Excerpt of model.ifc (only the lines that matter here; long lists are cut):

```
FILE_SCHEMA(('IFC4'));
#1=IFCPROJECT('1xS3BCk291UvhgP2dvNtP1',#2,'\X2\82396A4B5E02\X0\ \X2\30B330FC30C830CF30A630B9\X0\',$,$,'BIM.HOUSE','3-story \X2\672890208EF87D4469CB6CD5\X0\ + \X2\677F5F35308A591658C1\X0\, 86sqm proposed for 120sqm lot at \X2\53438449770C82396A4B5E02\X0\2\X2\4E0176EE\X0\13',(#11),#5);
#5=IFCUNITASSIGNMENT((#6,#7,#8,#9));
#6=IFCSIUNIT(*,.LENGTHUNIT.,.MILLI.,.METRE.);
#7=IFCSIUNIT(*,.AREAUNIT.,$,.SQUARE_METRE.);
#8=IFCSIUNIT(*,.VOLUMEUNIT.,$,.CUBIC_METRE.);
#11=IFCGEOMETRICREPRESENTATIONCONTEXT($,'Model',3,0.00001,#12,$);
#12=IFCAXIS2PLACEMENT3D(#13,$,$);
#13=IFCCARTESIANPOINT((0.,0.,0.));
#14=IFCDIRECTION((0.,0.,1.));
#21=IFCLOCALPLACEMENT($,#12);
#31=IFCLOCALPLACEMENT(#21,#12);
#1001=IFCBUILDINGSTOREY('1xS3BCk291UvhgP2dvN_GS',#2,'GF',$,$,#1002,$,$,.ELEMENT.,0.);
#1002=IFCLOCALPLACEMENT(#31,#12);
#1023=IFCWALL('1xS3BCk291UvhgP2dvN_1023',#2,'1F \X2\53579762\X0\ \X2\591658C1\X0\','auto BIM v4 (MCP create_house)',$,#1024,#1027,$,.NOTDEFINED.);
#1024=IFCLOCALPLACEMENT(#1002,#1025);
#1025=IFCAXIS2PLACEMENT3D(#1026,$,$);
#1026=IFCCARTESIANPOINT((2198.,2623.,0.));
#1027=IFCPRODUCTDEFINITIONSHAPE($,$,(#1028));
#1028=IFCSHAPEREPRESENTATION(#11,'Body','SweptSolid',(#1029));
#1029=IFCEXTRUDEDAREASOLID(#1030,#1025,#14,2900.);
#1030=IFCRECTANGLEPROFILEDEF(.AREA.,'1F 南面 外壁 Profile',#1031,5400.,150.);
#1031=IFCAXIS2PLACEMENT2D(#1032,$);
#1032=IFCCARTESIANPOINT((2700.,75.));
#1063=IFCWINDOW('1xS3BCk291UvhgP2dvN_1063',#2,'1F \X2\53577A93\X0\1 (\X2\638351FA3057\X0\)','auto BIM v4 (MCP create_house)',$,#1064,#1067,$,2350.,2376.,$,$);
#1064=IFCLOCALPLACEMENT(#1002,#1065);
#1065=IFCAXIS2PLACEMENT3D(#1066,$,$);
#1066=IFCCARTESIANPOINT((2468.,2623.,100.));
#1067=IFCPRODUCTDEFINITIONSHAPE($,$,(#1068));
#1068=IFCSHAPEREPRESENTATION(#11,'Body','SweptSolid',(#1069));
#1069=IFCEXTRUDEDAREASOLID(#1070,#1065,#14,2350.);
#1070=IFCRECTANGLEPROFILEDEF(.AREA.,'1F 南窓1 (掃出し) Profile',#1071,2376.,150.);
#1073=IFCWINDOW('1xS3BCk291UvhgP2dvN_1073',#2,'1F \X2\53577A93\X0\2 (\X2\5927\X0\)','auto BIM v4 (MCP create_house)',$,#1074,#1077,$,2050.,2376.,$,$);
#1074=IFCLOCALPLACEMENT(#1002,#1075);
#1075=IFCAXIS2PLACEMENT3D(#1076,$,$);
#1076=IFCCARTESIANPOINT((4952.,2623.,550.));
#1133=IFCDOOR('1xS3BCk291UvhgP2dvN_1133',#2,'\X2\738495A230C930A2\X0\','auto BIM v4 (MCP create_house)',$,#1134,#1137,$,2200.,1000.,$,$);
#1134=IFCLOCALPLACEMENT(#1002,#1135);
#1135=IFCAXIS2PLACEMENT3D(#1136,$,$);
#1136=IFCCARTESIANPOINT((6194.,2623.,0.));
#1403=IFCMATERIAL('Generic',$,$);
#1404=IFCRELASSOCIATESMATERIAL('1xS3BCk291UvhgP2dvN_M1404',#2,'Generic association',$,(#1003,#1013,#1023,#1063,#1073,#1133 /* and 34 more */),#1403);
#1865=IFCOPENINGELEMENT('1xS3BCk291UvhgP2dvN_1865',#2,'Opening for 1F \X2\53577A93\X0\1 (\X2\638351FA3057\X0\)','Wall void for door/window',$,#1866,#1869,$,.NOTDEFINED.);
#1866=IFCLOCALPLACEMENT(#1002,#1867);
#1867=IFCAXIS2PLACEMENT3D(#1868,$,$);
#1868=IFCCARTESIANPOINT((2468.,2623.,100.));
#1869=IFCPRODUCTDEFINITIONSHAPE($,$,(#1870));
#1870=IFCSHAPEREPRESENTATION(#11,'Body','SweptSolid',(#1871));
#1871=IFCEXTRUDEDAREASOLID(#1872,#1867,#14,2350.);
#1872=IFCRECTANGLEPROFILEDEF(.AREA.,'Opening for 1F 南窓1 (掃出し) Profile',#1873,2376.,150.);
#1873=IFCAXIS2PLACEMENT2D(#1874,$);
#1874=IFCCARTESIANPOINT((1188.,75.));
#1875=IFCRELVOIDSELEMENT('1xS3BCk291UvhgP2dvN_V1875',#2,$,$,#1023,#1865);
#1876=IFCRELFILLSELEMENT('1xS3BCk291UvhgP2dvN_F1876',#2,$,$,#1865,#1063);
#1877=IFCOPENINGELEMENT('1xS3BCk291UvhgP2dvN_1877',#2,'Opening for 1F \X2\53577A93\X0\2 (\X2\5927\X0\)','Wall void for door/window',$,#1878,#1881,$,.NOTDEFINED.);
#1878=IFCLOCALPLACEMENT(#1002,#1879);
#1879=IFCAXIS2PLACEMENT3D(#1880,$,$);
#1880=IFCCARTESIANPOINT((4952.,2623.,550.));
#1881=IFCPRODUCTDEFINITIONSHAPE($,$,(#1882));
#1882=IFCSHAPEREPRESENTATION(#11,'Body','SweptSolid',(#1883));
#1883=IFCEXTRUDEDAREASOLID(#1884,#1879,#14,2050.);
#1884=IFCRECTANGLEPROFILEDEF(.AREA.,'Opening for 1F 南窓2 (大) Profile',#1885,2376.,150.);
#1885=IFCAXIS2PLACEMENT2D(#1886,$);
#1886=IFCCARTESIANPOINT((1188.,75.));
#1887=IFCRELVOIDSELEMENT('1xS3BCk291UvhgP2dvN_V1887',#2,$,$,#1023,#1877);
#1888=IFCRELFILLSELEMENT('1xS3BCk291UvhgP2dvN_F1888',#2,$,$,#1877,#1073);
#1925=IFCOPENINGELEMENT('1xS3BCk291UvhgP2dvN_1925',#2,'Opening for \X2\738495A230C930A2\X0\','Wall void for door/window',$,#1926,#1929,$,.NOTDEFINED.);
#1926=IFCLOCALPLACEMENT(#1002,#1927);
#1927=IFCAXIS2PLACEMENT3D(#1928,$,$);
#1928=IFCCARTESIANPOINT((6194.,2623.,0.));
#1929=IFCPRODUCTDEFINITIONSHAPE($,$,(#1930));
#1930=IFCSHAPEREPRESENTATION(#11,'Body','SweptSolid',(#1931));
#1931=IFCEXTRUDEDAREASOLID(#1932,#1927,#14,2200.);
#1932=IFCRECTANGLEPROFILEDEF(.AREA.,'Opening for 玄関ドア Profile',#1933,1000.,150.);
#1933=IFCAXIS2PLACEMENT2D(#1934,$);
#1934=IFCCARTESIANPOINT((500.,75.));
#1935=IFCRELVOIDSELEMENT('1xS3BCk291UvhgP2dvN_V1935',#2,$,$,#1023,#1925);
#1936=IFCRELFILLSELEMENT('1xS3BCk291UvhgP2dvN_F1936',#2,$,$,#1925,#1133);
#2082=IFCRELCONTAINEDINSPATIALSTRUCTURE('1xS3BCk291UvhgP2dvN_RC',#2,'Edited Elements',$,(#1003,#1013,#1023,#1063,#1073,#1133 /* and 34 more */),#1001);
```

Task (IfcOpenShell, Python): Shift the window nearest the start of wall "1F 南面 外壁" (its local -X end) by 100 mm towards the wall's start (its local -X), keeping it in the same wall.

```python
import ifcopenshell
import ifcopenshell.api.geometry
import ifcopenshell.util.placement
import ifcopenshell.util.unit

model = ifcopenshell.open("model.ifc")
unit_scale = ifcopenshell.util.unit.calculate_unit_scale(model)

window = model.by_guid("1xS3BCk291UvhgP2dvN_1063")
opening = window.FillsVoids[0].RelatingOpeningElement
wall = opening.VoidsElements[0].RelatingBuildingElement

wall_matrix = ifcopenshell.util.placement.get_local_placement(wall.ObjectPlacement)
shift = wall_matrix[:3, 0] * -0.1 / unit_scale
before = ifcopenshell.util.placement.get_local_placement(window.ObjectPlacement)[:3, 3].copy()

# The window is not placed relative to its opening, so move both.
for product in (opening, window):
    matrix = ifcopenshell.util.placement.get_local_placement(product.ObjectPlacement)
    matrix[:3, 3] += shift
    ifcopenshell.api.geometry.edit_object_placement(model, product=product, matrix=matrix, is_si=False)

after = ifcopenshell.util.placement.get_local_placement(window.ObjectPlacement)[:3, 3]
print("window moved by", (after - before).round(3) + 0.0)

model.write("model_rev.ifc")
```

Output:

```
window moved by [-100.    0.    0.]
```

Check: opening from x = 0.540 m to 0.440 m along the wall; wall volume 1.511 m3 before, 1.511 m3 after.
